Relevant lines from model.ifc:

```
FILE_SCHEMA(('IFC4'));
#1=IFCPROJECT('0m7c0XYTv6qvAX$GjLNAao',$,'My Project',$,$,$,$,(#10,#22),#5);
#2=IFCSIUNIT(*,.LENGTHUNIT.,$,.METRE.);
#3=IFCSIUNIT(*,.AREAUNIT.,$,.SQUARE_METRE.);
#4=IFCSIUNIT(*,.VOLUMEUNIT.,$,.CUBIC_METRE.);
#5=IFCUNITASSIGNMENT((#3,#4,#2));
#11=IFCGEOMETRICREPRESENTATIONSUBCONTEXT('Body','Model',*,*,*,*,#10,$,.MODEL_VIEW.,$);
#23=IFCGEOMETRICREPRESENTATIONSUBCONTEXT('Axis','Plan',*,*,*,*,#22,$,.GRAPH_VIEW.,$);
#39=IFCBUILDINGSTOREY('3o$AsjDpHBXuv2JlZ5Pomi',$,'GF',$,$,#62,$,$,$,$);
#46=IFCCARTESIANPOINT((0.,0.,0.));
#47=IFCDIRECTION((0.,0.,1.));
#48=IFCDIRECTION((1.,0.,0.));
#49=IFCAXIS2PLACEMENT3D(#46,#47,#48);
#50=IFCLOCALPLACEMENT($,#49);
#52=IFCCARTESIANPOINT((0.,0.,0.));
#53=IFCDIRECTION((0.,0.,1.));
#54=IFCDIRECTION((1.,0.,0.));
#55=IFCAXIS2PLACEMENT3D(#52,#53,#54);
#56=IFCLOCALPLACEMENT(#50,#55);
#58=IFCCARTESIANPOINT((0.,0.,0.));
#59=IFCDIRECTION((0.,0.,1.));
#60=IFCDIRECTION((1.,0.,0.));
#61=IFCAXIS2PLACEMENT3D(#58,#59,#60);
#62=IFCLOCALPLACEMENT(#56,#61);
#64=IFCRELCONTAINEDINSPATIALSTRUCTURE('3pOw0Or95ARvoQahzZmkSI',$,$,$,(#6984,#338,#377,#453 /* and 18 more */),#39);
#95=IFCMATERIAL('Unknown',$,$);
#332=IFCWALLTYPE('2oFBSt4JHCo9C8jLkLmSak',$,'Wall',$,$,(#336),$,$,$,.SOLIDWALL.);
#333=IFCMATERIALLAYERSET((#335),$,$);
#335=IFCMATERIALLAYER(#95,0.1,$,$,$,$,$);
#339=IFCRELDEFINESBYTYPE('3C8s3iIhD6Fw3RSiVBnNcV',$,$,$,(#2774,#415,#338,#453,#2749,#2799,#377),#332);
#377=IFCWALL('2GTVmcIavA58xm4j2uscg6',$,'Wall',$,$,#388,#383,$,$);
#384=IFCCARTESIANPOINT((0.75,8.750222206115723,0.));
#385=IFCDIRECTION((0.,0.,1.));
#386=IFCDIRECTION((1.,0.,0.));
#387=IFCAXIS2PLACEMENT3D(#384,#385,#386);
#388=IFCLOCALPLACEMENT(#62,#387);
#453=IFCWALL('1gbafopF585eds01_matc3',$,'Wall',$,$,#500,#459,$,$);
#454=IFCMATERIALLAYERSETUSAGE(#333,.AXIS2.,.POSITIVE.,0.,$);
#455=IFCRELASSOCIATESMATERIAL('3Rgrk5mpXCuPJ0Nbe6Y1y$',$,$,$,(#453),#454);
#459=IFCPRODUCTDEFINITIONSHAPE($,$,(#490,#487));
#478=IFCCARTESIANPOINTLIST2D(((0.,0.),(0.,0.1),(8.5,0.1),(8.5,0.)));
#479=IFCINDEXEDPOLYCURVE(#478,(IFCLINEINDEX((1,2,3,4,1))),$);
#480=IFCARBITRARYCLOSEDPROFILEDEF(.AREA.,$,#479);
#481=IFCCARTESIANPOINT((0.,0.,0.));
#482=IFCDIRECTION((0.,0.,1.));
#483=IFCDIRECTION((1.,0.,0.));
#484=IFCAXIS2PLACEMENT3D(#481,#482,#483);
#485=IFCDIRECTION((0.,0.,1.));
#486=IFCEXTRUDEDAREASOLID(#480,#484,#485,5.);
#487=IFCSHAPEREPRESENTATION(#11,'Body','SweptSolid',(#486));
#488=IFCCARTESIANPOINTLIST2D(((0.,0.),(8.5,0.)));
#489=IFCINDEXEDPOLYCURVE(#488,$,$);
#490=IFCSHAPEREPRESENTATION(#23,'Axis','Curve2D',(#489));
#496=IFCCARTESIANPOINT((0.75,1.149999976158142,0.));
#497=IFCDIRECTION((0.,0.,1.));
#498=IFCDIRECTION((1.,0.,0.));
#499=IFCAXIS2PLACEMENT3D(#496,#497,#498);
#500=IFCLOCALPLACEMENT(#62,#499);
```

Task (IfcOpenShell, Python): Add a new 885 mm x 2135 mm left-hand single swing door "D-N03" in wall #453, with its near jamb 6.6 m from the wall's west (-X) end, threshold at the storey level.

```python
import numpy as np
import ifcopenshell
import ifcopenshell.api.feature
import ifcopenshell.api.geometry
import ifcopenshell.api.root
import ifcopenshell.api.spatial
import ifcopenshell.geom
import ifcopenshell.util.element
import ifcopenshell.util.placement
import ifcopenshell.util.representation
import ifcopenshell.util.shape
import ifcopenshell.util.unit

model = ifcopenshell.open("model.ifc")
unit_scale = ifcopenshell.util.unit.calculate_unit_scale(model)
settings = ifcopenshell.geom.settings()


def volume(element):
    """Net volume in cubic metres, openings subtracted."""
    shape = ifcopenshell.geom.create_shape(settings, element)
    return ifcopenshell.util.shape.get_volume(shape.geometry)


wall = model.by_guid("1gbafopF585eds01_matc3")
storey = ifcopenshell.util.element.get_container(wall, ifc_class="IfcBuildingStorey")
context = ifcopenshell.util.representation.get_context(model, "Model", "Body", "MODEL_VIEW")
before = volume(wall)

width, height, from_end, sill = 0.885, 2.135, 6.6, 0.0  # metres

# The wall runs along its own X axis, and the end named is its -X end.
wall_shape = ifcopenshell.geom.create_shape(settings, wall)
x, y, z = ifcopenshell.util.shape.get_vertices(wall_shape.geometry).T
start = x.min() + from_end
face, thickness = float(y.min()), float(y.max() - y.min())
wall_matrix = ifcopenshell.util.placement.get_local_placement(wall.ObjectPlacement)
level = ifcopenshell.util.placement.get_local_placement(storey.ObjectPlacement)[2, 3]


def in_wall(x, y):
    """Placement at x, y metres in the wall's axes, at sill height."""
    matrix = wall_matrix.copy()
    matrix[:, 3] = wall_matrix @ np.array([x / unit_scale, y / unit_scale, 0.0, 1.0])
    matrix[2, 3] = level + sill / unit_scale
    return matrix


# Opening: a box that overshoots both wall faces by 50 mm.
opening = ifcopenshell.api.root.create_entity(model, ifc_class="IfcOpeningElement", predefined_type="OPENING")
box = ifcopenshell.api.geometry.add_wall_representation(
    model, context=context, length=width, height=height, thickness=thickness + 0.1
)
ifcopenshell.api.geometry.assign_representation(model, product=opening, representation=box)
ifcopenshell.api.geometry.edit_object_placement(model, product=opening, matrix=in_wall(start, face - 0.05), is_si=False)
ifcopenshell.api.feature.add_feature(model, feature=opening, element=wall)

door = ifcopenshell.api.root.create_entity(model, ifc_class="IfcDoor", name="D-N03", predefined_type="DOOR")
door.OverallWidth, door.OverallHeight = width / unit_scale, height / unit_scale
door.OperationType = "SINGLE_SWING_LEFT"
body = ifcopenshell.api.geometry.add_door_representation(
    model,
    context=context,
    overall_width=door.OverallWidth,
    overall_height=door.OverallHeight,
    operation_type="SINGLE_SWING_LEFT",
    lining_properties={"LiningDepth": thickness / unit_scale, "ThresholdDepth": thickness / unit_scale},
)
ifcopenshell.api.geometry.assign_representation(model, product=door, representation=body)
ifcopenshell.api.spatial.assign_container(model, products=[door], relating_structure=storey)
ifcopenshell.api.feature.add_filling(model, opening=opening, element=door)

# The lining spans the wall, so the door starts at the wall face.
ifcopenshell.api.geometry.edit_object_placement(model, product=door, matrix=in_wall(start, face), is_si=False)

after = volume(wall)

print(f"wall volume {before:.3f} -> {after:.3f} m3")

model.write("model_v2.ifc")
```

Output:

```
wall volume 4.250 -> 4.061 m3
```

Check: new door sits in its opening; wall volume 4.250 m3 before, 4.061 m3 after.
